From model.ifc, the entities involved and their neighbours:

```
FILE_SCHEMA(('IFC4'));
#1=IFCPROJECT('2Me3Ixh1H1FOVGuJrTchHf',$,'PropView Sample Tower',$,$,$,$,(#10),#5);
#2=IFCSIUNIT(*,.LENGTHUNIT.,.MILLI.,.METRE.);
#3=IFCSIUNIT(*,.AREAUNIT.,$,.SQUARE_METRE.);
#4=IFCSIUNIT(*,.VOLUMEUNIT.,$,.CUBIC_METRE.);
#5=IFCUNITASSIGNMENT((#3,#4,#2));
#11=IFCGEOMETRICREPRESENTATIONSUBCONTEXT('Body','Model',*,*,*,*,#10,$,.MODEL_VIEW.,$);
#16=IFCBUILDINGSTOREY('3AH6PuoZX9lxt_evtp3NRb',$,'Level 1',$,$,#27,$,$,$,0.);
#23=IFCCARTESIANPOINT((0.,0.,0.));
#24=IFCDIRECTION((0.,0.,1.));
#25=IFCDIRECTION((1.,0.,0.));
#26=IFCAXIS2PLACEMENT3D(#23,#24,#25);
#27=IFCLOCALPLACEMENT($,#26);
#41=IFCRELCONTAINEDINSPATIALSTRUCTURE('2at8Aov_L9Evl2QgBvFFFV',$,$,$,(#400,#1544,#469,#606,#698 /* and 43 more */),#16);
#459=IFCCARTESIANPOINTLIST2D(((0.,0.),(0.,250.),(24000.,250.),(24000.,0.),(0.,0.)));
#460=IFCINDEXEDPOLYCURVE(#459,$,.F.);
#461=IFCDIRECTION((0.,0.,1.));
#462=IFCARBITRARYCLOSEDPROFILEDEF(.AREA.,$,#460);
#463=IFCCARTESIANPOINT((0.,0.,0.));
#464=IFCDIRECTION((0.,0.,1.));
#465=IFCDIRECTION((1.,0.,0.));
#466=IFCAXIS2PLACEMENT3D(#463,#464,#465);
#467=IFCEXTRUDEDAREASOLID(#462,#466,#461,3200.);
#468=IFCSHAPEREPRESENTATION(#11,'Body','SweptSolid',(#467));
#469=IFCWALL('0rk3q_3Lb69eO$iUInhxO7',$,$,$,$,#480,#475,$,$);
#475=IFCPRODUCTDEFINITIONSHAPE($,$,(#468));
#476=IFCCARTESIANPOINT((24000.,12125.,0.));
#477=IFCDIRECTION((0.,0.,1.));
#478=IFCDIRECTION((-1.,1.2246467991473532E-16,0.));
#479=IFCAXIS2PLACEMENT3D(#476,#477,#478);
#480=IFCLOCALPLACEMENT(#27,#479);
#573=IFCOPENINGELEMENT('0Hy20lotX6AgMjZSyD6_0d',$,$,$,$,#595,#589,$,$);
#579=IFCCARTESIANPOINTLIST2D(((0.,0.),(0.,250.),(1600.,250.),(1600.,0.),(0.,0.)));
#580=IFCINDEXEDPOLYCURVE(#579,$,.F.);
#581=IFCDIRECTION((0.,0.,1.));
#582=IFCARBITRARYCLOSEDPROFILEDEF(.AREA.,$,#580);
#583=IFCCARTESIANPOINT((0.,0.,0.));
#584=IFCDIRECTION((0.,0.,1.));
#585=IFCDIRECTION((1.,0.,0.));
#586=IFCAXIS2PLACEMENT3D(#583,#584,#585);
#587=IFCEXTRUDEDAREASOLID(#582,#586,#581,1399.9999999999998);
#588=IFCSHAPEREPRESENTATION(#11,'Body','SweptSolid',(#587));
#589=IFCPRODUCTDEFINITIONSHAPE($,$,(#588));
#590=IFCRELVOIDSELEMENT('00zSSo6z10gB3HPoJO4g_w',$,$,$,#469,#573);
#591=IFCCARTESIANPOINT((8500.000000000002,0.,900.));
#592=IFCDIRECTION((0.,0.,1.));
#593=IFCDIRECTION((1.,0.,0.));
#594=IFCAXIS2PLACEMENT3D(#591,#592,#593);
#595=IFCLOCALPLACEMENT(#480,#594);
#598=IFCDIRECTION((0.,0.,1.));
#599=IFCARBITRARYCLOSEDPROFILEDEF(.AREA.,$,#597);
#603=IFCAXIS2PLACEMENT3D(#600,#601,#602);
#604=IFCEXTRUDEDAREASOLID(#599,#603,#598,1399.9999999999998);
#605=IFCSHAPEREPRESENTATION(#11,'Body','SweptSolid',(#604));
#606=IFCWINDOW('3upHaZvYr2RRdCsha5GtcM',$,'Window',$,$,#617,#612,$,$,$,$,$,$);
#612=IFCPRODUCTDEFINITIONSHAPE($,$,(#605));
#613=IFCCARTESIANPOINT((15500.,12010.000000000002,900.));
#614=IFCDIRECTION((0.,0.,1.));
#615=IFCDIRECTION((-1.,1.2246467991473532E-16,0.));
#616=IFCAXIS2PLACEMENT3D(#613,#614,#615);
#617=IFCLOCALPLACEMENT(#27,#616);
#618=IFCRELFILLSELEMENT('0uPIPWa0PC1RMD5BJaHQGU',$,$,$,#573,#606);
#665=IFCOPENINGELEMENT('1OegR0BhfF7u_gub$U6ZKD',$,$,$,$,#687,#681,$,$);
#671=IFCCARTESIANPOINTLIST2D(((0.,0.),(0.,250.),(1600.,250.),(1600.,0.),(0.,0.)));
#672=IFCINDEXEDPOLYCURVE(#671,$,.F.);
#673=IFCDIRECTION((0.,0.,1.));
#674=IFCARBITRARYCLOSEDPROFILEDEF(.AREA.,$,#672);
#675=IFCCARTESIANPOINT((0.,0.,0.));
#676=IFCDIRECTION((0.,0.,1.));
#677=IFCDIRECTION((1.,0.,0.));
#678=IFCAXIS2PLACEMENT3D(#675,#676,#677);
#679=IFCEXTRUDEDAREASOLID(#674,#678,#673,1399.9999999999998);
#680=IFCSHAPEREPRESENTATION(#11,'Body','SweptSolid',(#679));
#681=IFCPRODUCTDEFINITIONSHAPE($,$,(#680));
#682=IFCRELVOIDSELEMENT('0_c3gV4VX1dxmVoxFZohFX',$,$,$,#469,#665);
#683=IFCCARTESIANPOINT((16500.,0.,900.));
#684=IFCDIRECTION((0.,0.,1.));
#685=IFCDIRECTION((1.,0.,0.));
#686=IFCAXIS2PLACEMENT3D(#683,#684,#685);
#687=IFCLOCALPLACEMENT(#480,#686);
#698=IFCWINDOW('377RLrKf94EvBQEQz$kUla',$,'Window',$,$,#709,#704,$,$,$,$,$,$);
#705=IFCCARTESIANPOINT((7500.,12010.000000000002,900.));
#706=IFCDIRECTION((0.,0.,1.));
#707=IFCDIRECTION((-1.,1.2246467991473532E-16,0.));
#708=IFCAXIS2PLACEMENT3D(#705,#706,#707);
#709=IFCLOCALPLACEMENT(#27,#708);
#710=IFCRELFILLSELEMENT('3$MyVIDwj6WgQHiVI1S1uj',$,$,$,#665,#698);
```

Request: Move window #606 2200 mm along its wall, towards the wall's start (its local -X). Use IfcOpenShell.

```python
import ifcopenshell
import ifcopenshell.api.geometry
import ifcopenshell.util.placement
import ifcopenshell.util.unit

model = ifcopenshell.open("model.ifc")
unit_scale = ifcopenshell.util.unit.calculate_unit_scale(model)

window = model.by_id(606)
opening = window.FillsVoids[0].RelatingOpeningElement
wall = opening.VoidsElements[0].RelatingBuildingElement

wall_matrix = ifcopenshell.util.placement.get_local_placement(wall.ObjectPlacement)
shift = wall_matrix[:3, 0] * -2.2 / unit_scale
before = ifcopenshell.util.placement.get_local_placement(window.ObjectPlacement)[:3, 3].copy()

# The window is not placed relative to its opening, so move both.
for product in (opening, window):
    matrix = ifcopenshell.util.placement.get_local_placement(product.ObjectPlacement)
    matrix[:3, 3] += shift
    ifcopenshell.api.geometry.edit_object_placement(model, product=product, matrix=matrix, is_si=False)

after = ifcopenshell.util.placement.get_local_placement(window.ObjectPlacement)[:3, 3]
print("window moved by", (after - before).round(3) + 0.0)

model.write("model_v2.ifc")
```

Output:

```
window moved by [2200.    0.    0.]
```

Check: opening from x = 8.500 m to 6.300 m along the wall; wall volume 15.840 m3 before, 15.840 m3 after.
